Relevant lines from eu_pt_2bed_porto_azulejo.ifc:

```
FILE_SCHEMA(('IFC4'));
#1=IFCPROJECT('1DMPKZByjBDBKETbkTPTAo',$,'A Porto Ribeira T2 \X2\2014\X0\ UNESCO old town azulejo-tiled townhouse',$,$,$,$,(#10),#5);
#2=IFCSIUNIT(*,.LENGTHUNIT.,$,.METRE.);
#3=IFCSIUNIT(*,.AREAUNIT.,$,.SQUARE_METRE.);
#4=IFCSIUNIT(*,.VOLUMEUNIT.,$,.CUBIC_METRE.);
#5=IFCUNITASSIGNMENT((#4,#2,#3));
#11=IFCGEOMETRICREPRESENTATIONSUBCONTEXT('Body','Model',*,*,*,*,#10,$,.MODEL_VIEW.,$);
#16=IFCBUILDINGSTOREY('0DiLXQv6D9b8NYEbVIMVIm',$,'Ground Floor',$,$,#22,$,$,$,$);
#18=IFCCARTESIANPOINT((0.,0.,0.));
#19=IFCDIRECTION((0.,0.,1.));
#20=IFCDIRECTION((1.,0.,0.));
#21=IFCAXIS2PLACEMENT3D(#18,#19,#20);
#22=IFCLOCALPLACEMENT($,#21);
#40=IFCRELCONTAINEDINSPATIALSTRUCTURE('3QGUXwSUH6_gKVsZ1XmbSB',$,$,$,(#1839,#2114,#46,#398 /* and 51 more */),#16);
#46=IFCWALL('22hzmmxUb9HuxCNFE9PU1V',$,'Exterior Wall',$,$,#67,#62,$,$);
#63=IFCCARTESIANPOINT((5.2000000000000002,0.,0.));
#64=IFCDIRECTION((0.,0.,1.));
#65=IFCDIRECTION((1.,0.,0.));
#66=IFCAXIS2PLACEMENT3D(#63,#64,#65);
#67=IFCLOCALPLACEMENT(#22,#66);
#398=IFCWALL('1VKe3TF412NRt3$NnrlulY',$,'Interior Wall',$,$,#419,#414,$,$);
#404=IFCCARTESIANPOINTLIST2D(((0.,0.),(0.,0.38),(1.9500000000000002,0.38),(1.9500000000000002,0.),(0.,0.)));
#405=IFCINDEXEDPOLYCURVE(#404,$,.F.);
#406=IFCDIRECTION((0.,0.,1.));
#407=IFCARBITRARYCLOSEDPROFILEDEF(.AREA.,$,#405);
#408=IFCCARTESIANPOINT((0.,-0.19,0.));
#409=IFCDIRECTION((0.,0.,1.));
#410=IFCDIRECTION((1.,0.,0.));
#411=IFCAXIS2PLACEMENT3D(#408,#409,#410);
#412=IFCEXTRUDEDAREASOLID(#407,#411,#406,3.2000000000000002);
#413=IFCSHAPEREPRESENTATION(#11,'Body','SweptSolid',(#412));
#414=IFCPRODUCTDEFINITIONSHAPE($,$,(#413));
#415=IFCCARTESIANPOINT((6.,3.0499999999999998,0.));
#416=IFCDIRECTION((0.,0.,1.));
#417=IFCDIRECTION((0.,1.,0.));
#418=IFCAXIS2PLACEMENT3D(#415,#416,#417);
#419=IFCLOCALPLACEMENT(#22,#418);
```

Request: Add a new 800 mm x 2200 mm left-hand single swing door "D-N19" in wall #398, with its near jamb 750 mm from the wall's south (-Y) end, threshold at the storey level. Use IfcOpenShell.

```python
import numpy as np
import ifcopenshell
import ifcopenshell.api.feature
import ifcopenshell.api.geometry
import ifcopenshell.api.root
import ifcopenshell.api.spatial
import ifcopenshell.geom
import ifcopenshell.util.element
import ifcopenshell.util.placement
import ifcopenshell.util.representation
import ifcopenshell.util.shape
import ifcopenshell.util.unit

model = ifcopenshell.open("eu_pt_2bed_porto_azulejo.ifc")
unit_scale = ifcopenshell.util.unit.calculate_unit_scale(model)
settings = ifcopenshell.geom.settings()


def volume(element):
    """Net volume in cubic metres, openings subtracted."""
    shape = ifcopenshell.geom.create_shape(settings, element)
    return ifcopenshell.util.shape.get_volume(shape.geometry)


wall = model.by_guid("1VKe3TF412NRt3$NnrlulY")
storey = ifcopenshell.util.element.get_container(wall, ifc_class="IfcBuildingStorey")
context = ifcopenshell.util.representation.get_context(model, "Model", "Body", "MODEL_VIEW")
before = volume(wall)

width, height, from_end, sill = 0.8, 2.2, 0.75, 0.0  # metres

# The wall runs along its own X axis, and the end named is its -X end.
wall_shape = ifcopenshell.geom.create_shape(settings, wall)
x, y, z = ifcopenshell.util.shape.get_vertices(wall_shape.geometry).T
start = x.min() + from_end
face, thickness = float(y.min()), float(y.max() - y.min())
wall_matrix = ifcopenshell.util.placement.get_local_placement(wall.ObjectPlacement)
level = ifcopenshell.util.placement.get_local_placement(storey.ObjectPlacement)[2, 3]


def in_wall(x, y):
    """Placement at x, y metres in the wall's axes, at sill height."""
    matrix = wall_matrix.copy()
    matrix[:, 3] = wall_matrix @ np.array([x / unit_scale, y / unit_scale, 0.0, 1.0])
    matrix[2, 3] = level + sill / unit_scale
    return matrix


# Opening: a box that overshoots both wall faces by 50 mm.
opening = ifcopenshell.api.root.create_entity(model, ifc_class="IfcOpeningElement", predefined_type="OPENING")
box = ifcopenshell.api.geometry.add_wall_representation(
    model, context=context, length=width, height=height, thickness=thickness + 0.1
)
ifcopenshell.api.geometry.assign_representation(model, product=opening, representation=box)
ifcopenshell.api.geometry.edit_object_placement(model, product=opening, matrix=in_wall(start, face - 0.05), is_si=False)
ifcopenshell.api.feature.add_feature(model, feature=opening, element=wall)

door = ifcopenshell.api.root.create_entity(model, ifc_class="IfcDoor", name="D-N19", predefined_type="DOOR")
door.OverallWidth, door.OverallHeight = width / unit_scale, height / unit_scale
door.OperationType = "SINGLE_SWING_LEFT"
body = ifcopenshell.api.geometry.add_door_representation(
    model,
    context=context,
    overall_width=door.OverallWidth,
    overall_height=door.OverallHeight,
    operation_type="SINGLE_SWING_LEFT",
    lining_properties={"LiningDepth": thickness / unit_scale, "ThresholdDepth": thickness / unit_scale},
)
ifcopenshell.api.geometry.assign_representation(model, product=door, representation=body)
ifcopenshell.api.spatial.assign_container(model, products=[door], relating_structure=storey)
ifcopenshell.api.feature.add_filling(model, opening=opening, element=door)

# The lining spans the wall, so the door starts at the wall face.
ifcopenshell.api.geometry.edit_object_placement(model, product=door, matrix=in_wall(start, face), is_si=False)

after = volume(wall)

print(f"wall volume {before:.3f} -> {after:.3f} m3")

model.write("eu_pt_2bed_porto_azulejo_edited.ifc")
```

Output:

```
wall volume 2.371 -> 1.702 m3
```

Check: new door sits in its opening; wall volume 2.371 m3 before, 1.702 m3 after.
